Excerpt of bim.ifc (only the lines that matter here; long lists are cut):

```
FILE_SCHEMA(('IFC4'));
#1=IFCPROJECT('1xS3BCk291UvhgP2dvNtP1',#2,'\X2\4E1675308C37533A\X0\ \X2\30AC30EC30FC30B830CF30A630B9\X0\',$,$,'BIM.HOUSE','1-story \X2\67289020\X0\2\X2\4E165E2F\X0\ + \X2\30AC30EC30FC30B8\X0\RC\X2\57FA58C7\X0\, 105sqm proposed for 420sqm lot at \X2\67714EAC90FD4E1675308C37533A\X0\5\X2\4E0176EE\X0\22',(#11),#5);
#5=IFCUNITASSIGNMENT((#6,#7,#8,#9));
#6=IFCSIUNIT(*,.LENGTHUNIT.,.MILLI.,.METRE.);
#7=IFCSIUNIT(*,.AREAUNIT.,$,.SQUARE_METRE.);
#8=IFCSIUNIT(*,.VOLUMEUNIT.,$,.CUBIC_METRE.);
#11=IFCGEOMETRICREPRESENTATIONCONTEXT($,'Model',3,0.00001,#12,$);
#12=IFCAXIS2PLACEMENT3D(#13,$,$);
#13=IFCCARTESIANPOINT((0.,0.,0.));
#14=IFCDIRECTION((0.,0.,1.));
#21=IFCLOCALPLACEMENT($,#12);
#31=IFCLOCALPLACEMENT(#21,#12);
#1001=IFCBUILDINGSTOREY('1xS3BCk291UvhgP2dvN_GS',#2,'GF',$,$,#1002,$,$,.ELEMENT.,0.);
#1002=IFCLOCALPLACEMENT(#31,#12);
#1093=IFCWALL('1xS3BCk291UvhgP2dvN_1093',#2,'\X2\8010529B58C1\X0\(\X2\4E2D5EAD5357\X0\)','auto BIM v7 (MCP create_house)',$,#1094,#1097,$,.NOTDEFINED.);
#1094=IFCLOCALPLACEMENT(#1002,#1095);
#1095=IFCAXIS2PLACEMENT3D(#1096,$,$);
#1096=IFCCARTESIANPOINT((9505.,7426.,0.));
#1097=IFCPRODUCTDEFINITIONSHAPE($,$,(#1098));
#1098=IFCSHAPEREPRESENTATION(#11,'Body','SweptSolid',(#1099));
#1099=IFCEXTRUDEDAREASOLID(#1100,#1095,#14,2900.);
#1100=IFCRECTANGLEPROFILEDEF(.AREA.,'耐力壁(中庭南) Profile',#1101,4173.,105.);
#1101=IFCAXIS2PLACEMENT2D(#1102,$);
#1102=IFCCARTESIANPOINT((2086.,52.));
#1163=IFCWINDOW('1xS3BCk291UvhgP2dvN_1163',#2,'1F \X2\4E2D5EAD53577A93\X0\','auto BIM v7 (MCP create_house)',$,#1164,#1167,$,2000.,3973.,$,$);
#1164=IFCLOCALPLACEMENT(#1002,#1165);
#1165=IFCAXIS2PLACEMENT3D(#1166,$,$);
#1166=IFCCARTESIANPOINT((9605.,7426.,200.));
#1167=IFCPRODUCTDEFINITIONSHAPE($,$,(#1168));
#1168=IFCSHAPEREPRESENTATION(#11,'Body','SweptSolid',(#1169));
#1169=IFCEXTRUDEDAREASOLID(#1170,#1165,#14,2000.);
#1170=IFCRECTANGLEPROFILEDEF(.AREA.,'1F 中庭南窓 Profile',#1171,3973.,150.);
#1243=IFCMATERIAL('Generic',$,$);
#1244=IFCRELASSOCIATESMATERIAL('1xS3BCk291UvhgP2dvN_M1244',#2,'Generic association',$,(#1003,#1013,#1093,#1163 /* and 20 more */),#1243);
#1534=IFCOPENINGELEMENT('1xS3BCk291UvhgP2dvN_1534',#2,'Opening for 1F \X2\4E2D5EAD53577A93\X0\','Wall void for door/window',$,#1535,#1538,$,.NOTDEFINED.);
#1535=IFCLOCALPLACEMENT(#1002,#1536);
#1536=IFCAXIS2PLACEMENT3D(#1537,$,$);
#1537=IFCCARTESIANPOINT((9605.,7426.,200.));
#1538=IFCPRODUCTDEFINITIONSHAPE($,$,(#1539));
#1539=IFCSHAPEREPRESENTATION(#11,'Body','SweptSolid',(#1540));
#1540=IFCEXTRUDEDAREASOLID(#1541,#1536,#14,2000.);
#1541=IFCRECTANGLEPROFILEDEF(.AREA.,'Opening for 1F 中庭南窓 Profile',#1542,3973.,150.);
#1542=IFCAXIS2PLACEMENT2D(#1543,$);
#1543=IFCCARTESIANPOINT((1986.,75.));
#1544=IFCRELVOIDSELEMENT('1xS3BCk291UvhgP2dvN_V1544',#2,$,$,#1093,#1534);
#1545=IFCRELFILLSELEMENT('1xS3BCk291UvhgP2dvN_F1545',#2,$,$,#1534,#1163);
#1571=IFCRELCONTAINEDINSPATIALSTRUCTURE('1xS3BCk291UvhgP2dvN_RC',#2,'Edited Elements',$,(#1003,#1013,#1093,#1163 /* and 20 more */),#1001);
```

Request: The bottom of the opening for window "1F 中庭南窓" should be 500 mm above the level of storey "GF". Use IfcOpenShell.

```python
import numpy as np
import ifcopenshell
import ifcopenshell.api.geometry
import ifcopenshell.geom
import ifcopenshell.util.element
import ifcopenshell.util.placement
import ifcopenshell.util.shape
import ifcopenshell.util.unit

model = ifcopenshell.open("bim.ifc")
unit_scale = ifcopenshell.util.unit.calculate_unit_scale(model)

window = model.by_guid("1xS3BCk291UvhgP2dvN_1163")
opening = window.FillsVoids[0].RelatingOpeningElement
storey = ifcopenshell.util.element.get_container(window, ifc_class="IfcBuildingStorey")
level = ifcopenshell.util.placement.get_local_placement(storey.ObjectPlacement)[2, 3]

# The opening's origin need not be at the sill, so measure its lowest point.
shape = ifcopenshell.geom.create_shape(ifcopenshell.geom.settings(), opening)
bottom = ifcopenshell.util.shape.get_shape_bottom_elevation(shape, shape.geometry) / unit_scale
dz = level + 0.5 / unit_scale - bottom

shift = np.array([0.0, 0.0, dz])
# The window is not placed relative to its opening, so move both.
for product in (opening, window):
    matrix = ifcopenshell.util.placement.get_local_placement(product.ObjectPlacement)
    matrix[:3, 3] += shift
    ifcopenshell.api.geometry.edit_object_placement(model, product=product, matrix=matrix, is_si=False)

print(f"moved by {dz * unit_scale:+.3f} m")

model.write("bim_updated.ifc")
```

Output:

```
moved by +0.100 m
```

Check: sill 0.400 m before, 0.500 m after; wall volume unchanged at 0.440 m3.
